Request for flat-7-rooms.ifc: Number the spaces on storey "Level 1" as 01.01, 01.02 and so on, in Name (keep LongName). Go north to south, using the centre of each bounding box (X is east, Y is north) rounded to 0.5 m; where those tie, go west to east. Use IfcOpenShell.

First a look at what the model holds.

```python
import ifcopenshell
import ifcopenshell.util.element
import ifcopenshell.util.placement

model = ifcopenshell.open("flat-7-rooms.ifc")
print(model.schema)
storey = next(s for s in model.by_type("IfcBuildingStorey") if s.Name == "Level 1")
spaces = [e for e in ifcopenshell.util.element.get_decomposition(storey) if e.is_a("IfcSpace")]
for e in sorted(spaces, key=lambda e: e.id()):
    origin = ifcopenshell.util.placement.get_local_placement(e.ObjectPlacement)[:3, 3]
    print(e.id(), e.Name, e.LongName, origin.round(2) + 0.0, sep=" | ")
```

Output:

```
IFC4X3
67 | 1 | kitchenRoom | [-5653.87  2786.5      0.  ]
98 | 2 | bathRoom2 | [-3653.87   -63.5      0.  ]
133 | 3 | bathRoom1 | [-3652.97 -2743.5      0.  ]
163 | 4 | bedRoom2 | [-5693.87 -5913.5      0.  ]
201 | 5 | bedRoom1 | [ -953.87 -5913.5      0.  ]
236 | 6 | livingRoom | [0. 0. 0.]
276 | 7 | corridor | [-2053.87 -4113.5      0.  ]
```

```python
import ifcopenshell
import ifcopenshell.geom
import ifcopenshell.util.element
import ifcopenshell.util.shape

model = ifcopenshell.open("flat-7-rooms.ifc")
settings = ifcopenshell.geom.settings()
settings.set("use-world-coords", True)


def centre(element):
    shape = ifcopenshell.geom.create_shape(settings, element)
    return ifcopenshell.util.shape.get_bbox_centroid(shape.geometry)


storey = next(s for s in model.by_type("IfcBuildingStorey") if s.Name == "Level 1")
spaces = [e for e in ifcopenshell.util.element.get_decomposition(storey) if e.is_a("IfcSpace")]

# Insertion points can sit at a corner or the storey origin, so sort by the geometry (in metres).
centres = {e: centre(e) for e in spaces}
spaces.sort(key=lambda e: (-round(centres[e][1] / 0.5), centres[e][0]))

for i, e in enumerate(spaces, start=1):
    number = f"01.{i:02d}"
    e.Name = number
    print(e.id(), number)

model.write("flat-7-rooms_rev.ifc")
```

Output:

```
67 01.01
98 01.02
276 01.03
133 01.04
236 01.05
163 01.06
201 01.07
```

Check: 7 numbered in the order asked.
